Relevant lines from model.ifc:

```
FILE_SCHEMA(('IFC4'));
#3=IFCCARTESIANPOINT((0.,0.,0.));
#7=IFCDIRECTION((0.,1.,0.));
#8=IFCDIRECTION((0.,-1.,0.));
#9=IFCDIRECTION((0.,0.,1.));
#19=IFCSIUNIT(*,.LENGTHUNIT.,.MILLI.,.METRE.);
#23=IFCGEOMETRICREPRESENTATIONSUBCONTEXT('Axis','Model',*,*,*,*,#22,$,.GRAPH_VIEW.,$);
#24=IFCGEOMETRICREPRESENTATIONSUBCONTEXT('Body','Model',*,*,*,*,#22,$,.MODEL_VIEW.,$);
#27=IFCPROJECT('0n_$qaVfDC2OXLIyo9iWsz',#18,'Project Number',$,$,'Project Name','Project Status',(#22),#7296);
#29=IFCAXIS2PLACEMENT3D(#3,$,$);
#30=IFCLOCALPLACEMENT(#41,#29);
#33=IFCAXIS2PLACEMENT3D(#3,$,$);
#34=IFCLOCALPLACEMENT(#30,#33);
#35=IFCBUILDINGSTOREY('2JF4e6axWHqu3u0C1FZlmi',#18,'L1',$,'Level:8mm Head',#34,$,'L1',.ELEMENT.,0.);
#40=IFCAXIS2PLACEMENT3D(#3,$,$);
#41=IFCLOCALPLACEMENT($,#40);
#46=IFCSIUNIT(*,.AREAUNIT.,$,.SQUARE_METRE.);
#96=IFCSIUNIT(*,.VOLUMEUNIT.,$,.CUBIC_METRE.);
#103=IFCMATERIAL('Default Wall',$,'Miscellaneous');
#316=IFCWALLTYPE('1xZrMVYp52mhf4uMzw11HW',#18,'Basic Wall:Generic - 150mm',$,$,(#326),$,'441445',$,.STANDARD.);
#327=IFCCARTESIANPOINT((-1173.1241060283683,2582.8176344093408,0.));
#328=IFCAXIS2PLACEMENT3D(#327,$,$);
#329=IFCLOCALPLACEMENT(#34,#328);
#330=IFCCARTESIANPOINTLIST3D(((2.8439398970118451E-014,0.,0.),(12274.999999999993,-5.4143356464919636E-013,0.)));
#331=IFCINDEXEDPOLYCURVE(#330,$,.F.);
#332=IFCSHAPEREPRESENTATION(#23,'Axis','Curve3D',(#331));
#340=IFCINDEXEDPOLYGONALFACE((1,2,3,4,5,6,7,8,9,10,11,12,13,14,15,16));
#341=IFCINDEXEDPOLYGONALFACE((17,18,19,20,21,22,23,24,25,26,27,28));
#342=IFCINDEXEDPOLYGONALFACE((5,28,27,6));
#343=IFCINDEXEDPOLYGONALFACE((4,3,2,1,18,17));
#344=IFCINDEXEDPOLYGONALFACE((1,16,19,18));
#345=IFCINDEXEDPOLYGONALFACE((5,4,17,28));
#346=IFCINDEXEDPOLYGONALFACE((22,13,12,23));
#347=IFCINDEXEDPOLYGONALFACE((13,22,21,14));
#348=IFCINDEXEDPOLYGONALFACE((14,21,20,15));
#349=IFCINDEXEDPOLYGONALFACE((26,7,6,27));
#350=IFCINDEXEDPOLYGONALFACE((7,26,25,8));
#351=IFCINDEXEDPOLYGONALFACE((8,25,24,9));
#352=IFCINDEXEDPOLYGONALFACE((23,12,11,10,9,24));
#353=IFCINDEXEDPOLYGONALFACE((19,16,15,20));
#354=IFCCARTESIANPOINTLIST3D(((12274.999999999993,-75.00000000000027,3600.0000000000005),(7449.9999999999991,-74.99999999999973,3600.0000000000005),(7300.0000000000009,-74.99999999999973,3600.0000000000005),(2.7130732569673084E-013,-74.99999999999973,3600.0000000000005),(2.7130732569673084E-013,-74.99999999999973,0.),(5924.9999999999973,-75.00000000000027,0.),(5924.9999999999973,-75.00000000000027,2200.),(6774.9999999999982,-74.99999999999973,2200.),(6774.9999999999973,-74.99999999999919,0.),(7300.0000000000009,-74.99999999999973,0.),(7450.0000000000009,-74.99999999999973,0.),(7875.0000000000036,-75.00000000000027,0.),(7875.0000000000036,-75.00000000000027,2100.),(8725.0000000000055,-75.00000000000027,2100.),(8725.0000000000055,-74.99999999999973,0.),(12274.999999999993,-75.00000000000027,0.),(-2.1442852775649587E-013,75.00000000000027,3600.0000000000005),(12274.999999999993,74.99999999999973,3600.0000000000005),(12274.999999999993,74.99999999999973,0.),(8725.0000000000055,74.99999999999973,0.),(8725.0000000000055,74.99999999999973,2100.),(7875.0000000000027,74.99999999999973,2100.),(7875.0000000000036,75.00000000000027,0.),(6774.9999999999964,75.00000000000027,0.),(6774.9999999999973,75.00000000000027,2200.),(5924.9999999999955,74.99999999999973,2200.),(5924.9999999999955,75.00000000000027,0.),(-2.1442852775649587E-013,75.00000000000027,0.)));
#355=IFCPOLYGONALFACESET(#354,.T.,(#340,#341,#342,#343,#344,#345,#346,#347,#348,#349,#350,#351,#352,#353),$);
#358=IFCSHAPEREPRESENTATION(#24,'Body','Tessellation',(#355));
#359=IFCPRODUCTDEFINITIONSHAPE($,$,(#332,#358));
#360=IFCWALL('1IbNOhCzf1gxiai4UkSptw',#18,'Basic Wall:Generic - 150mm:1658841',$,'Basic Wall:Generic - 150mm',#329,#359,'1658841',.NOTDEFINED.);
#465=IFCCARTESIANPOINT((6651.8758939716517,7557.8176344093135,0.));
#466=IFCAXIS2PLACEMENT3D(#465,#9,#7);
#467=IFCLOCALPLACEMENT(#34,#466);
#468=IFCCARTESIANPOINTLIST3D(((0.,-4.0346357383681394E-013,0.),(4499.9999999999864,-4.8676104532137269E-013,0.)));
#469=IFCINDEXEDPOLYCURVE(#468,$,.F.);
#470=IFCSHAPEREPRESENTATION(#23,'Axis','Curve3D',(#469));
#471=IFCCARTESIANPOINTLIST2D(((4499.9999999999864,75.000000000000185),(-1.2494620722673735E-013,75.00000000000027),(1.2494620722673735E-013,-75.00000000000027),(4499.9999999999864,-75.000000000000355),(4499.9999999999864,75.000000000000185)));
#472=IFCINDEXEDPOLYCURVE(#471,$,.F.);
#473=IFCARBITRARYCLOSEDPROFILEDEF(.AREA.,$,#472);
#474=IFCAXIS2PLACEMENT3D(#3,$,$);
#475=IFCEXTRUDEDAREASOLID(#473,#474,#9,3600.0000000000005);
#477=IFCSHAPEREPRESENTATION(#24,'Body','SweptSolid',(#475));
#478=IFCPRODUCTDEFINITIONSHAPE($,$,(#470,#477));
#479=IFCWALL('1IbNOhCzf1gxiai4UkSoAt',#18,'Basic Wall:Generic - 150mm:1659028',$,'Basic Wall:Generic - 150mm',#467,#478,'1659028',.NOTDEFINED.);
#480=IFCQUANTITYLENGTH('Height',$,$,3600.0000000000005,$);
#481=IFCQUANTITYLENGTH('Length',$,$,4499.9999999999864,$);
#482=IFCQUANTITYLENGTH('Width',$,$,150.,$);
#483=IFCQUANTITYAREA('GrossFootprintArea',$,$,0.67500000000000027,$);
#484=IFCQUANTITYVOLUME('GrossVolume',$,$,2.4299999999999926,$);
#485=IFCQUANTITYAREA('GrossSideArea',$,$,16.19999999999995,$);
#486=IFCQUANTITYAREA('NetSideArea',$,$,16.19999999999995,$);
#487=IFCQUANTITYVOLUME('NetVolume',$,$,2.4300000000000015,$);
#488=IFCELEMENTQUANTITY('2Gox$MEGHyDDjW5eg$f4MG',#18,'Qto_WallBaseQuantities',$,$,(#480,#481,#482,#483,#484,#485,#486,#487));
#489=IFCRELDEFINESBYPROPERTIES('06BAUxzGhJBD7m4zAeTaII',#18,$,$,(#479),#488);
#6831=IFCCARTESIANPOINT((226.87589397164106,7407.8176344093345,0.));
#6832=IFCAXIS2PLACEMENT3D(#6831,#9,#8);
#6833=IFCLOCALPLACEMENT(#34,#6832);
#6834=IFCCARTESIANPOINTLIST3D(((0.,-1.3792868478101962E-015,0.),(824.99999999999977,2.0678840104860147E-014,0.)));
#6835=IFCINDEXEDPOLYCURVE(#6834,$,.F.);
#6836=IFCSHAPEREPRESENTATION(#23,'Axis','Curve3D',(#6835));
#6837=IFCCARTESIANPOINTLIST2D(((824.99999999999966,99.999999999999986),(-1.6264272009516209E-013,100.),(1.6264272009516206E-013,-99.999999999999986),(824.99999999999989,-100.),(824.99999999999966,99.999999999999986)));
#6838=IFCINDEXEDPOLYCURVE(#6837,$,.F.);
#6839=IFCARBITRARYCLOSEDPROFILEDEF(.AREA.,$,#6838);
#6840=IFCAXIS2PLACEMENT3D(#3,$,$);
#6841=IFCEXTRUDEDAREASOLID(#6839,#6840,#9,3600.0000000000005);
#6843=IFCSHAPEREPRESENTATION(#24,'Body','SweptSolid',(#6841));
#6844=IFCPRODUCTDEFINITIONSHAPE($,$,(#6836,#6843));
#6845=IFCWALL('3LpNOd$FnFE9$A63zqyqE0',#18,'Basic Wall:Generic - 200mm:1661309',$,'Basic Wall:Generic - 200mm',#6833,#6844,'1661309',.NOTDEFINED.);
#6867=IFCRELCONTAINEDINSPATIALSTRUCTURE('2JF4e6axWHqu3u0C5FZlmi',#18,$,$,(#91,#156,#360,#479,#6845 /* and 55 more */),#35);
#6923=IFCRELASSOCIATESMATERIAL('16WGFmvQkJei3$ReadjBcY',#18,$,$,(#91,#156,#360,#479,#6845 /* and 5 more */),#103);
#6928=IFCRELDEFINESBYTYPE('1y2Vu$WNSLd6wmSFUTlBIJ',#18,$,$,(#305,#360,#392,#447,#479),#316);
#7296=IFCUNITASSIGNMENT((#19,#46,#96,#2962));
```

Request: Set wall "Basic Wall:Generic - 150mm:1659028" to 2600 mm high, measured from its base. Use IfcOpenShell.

```python
import ifcopenshell
import ifcopenshell.api.pset
import ifcopenshell.geom
import ifcopenshell.util.element
import ifcopenshell.util.representation
import ifcopenshell.util.shape
import ifcopenshell.util.unit

model = ifcopenshell.open("model.ifc")
unit_scale = ifcopenshell.util.unit.calculate_unit_scale(model)
area_scale = ifcopenshell.util.unit.calculate_unit_scale(model, "AREAUNIT")
volume_scale = ifcopenshell.util.unit.calculate_unit_scale(model, "VOLUMEUNIT")
settings = ifcopenshell.geom.settings()


def volume(element):
    """Net volume in cubic metres, openings subtracted."""
    shape = ifcopenshell.geom.create_shape(settings, element)
    return ifcopenshell.util.shape.get_volume(shape.geometry)


wall = model.by_id(479)
before = volume(wall)

body = ifcopenshell.util.representation.get_representation(wall, "Model", "Body")
solid = body.Items[0]
old_height = solid.Depth
solid.Depth = 2600.0
after = volume(wall)
thickness = 0.15  # wall thickness in metres

# Update the stored height, areas and volumes.
qto = model.by_id(ifcopenshell.util.element.get_pset(wall, "Qto_WallBaseQuantities", should_inherit=False)["id"])
ifcopenshell.api.pset.edit_qto(model, qto=qto, properties={
    "Height": solid.Depth,
    "GrossVolume": ifcopenshell.util.element.get_pset(wall, "Qto_WallBaseQuantities", "GrossVolume") * solid.Depth / old_height,
    "GrossSideArea": ifcopenshell.util.element.get_pset(wall, "Qto_WallBaseQuantities", "GrossSideArea") * solid.Depth / old_height,
    "NetSideArea": after / thickness / area_scale,
    "NetVolume": after / volume_scale,
})

print(f"height {old_height:g} -> {solid.Depth:g}, volume {before:.3f} -> {after:.3f} m3")

model.write("model_updated.ifc")
```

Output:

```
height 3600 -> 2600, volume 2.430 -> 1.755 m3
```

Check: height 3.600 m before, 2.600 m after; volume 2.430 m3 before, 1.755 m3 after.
